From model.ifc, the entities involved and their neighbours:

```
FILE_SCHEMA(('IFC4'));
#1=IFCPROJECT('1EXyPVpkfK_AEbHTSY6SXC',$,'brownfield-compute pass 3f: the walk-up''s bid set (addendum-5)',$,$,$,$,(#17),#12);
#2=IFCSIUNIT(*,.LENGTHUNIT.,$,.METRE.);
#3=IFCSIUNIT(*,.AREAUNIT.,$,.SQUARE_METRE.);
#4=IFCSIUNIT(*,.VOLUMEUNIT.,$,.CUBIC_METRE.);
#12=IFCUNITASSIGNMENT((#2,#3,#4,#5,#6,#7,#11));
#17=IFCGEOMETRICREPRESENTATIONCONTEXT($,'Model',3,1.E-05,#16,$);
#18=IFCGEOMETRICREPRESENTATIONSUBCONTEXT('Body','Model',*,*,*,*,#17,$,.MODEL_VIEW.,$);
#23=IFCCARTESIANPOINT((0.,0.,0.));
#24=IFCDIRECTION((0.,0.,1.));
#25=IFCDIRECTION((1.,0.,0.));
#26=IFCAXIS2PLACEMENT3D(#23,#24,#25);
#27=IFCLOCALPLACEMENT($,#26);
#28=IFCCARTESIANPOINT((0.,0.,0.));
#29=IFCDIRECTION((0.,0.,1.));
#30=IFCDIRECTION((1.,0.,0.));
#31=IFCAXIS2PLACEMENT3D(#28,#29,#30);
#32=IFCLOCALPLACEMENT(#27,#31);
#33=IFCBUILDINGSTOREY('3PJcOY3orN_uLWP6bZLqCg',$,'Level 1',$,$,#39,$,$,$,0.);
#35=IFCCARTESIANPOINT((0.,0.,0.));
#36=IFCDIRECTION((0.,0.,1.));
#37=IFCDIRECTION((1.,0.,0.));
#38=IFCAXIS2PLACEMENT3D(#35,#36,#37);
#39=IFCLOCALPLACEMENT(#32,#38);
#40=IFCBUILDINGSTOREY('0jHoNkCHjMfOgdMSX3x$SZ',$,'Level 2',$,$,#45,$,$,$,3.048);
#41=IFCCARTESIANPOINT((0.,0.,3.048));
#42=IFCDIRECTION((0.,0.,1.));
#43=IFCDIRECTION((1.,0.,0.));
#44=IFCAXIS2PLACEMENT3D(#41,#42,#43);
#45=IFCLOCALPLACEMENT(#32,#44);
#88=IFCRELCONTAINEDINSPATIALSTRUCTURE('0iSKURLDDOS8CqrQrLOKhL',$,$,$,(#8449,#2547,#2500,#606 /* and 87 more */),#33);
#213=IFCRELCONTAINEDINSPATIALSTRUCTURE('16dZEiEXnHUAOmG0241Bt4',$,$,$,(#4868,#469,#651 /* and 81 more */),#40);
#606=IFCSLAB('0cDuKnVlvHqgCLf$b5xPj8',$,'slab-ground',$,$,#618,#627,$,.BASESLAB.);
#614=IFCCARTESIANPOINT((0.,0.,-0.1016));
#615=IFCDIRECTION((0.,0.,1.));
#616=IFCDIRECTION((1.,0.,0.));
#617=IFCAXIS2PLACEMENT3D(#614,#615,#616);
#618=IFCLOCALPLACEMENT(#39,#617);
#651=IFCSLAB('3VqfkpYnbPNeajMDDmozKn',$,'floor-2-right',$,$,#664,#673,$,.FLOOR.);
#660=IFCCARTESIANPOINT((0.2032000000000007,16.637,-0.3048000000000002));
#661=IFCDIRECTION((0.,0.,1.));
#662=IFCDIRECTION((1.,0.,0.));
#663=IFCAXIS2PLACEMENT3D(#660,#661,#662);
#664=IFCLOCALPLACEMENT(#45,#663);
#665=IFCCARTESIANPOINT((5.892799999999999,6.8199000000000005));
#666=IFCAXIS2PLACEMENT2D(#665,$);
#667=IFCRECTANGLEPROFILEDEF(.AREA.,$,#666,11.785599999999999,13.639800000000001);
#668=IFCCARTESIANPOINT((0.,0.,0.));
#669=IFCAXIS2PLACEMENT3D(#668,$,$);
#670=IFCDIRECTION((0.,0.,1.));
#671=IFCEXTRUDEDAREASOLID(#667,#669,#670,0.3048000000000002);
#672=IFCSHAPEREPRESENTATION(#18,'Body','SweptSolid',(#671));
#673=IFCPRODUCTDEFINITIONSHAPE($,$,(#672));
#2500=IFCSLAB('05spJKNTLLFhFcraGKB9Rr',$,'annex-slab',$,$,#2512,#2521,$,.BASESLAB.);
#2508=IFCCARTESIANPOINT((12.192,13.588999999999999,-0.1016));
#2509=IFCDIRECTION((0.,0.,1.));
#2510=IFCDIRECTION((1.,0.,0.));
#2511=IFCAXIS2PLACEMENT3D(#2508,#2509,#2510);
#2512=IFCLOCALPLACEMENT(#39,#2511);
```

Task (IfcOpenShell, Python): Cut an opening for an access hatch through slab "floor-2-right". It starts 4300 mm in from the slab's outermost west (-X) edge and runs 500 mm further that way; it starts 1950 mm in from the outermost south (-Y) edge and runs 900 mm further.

```python
import numpy as np
import ifcopenshell
import ifcopenshell.api.feature
import ifcopenshell.api.geometry
import ifcopenshell.api.root
import ifcopenshell.geom
import ifcopenshell.util.placement
import ifcopenshell.util.representation
import ifcopenshell.util.shape
import ifcopenshell.util.unit

model = ifcopenshell.open("model.ifc")
unit_scale = ifcopenshell.util.unit.calculate_unit_scale(model)
settings = ifcopenshell.geom.settings()


def volume(element):
    """Net volume in cubic metres, openings subtracted."""
    shape = ifcopenshell.geom.create_shape(settings, element)
    return ifcopenshell.util.shape.get_volume(shape.geometry)


slab = model.by_guid("3VqfkpYnbPNeajMDDmozKn")
before = volume(slab)

# Extent in the slab's own axes, in metres. The edges named are its -X and -Y sides.
slab_shape = ifcopenshell.geom.create_shape(settings, slab)
vertices = ifcopenshell.util.shape.get_vertices(slab_shape.geometry)
x_min, y_min, bottom = vertices.min(axis=0)
top = vertices[:, 2].max()

opening = ifcopenshell.api.root.create_entity(model, ifc_class="IfcOpeningElement", name="Access hatch opening", predefined_type="OPENING")
context = ifcopenshell.util.representation.get_context(model, "Model", "Body", "MODEL_VIEW")
width, depth = 0.5, 0.9
outline = [(0.0, 0.0), (width, 0.0), (width, depth), (0.0, depth), (0.0, 0.0)]
# Overshoot both faces by 50 mm so the cut is clean.
shape = ifcopenshell.api.geometry.add_slab_representation(
    model, context=context, depth=top - bottom + 0.1, polyline=outline
)
ifcopenshell.api.geometry.assign_representation(model, product=opening, representation=shape)

matrix = ifcopenshell.util.placement.get_local_placement(slab.ObjectPlacement)
matrix[:, 3] = matrix @ np.append(np.array([x_min + 4.3, y_min + 1.95, bottom - 0.05]) / unit_scale, 1.0)
ifcopenshell.api.geometry.edit_object_placement(model, product=opening, matrix=matrix, is_si=False)
ifcopenshell.api.feature.add_feature(model, feature=opening, element=slab)

after = volume(slab)

print(f"slab volume {before:.3f} -> {after:.3f} m3")

model.write("model_rev.ifc")
```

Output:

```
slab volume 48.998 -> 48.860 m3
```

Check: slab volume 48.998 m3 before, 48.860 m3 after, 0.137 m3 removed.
